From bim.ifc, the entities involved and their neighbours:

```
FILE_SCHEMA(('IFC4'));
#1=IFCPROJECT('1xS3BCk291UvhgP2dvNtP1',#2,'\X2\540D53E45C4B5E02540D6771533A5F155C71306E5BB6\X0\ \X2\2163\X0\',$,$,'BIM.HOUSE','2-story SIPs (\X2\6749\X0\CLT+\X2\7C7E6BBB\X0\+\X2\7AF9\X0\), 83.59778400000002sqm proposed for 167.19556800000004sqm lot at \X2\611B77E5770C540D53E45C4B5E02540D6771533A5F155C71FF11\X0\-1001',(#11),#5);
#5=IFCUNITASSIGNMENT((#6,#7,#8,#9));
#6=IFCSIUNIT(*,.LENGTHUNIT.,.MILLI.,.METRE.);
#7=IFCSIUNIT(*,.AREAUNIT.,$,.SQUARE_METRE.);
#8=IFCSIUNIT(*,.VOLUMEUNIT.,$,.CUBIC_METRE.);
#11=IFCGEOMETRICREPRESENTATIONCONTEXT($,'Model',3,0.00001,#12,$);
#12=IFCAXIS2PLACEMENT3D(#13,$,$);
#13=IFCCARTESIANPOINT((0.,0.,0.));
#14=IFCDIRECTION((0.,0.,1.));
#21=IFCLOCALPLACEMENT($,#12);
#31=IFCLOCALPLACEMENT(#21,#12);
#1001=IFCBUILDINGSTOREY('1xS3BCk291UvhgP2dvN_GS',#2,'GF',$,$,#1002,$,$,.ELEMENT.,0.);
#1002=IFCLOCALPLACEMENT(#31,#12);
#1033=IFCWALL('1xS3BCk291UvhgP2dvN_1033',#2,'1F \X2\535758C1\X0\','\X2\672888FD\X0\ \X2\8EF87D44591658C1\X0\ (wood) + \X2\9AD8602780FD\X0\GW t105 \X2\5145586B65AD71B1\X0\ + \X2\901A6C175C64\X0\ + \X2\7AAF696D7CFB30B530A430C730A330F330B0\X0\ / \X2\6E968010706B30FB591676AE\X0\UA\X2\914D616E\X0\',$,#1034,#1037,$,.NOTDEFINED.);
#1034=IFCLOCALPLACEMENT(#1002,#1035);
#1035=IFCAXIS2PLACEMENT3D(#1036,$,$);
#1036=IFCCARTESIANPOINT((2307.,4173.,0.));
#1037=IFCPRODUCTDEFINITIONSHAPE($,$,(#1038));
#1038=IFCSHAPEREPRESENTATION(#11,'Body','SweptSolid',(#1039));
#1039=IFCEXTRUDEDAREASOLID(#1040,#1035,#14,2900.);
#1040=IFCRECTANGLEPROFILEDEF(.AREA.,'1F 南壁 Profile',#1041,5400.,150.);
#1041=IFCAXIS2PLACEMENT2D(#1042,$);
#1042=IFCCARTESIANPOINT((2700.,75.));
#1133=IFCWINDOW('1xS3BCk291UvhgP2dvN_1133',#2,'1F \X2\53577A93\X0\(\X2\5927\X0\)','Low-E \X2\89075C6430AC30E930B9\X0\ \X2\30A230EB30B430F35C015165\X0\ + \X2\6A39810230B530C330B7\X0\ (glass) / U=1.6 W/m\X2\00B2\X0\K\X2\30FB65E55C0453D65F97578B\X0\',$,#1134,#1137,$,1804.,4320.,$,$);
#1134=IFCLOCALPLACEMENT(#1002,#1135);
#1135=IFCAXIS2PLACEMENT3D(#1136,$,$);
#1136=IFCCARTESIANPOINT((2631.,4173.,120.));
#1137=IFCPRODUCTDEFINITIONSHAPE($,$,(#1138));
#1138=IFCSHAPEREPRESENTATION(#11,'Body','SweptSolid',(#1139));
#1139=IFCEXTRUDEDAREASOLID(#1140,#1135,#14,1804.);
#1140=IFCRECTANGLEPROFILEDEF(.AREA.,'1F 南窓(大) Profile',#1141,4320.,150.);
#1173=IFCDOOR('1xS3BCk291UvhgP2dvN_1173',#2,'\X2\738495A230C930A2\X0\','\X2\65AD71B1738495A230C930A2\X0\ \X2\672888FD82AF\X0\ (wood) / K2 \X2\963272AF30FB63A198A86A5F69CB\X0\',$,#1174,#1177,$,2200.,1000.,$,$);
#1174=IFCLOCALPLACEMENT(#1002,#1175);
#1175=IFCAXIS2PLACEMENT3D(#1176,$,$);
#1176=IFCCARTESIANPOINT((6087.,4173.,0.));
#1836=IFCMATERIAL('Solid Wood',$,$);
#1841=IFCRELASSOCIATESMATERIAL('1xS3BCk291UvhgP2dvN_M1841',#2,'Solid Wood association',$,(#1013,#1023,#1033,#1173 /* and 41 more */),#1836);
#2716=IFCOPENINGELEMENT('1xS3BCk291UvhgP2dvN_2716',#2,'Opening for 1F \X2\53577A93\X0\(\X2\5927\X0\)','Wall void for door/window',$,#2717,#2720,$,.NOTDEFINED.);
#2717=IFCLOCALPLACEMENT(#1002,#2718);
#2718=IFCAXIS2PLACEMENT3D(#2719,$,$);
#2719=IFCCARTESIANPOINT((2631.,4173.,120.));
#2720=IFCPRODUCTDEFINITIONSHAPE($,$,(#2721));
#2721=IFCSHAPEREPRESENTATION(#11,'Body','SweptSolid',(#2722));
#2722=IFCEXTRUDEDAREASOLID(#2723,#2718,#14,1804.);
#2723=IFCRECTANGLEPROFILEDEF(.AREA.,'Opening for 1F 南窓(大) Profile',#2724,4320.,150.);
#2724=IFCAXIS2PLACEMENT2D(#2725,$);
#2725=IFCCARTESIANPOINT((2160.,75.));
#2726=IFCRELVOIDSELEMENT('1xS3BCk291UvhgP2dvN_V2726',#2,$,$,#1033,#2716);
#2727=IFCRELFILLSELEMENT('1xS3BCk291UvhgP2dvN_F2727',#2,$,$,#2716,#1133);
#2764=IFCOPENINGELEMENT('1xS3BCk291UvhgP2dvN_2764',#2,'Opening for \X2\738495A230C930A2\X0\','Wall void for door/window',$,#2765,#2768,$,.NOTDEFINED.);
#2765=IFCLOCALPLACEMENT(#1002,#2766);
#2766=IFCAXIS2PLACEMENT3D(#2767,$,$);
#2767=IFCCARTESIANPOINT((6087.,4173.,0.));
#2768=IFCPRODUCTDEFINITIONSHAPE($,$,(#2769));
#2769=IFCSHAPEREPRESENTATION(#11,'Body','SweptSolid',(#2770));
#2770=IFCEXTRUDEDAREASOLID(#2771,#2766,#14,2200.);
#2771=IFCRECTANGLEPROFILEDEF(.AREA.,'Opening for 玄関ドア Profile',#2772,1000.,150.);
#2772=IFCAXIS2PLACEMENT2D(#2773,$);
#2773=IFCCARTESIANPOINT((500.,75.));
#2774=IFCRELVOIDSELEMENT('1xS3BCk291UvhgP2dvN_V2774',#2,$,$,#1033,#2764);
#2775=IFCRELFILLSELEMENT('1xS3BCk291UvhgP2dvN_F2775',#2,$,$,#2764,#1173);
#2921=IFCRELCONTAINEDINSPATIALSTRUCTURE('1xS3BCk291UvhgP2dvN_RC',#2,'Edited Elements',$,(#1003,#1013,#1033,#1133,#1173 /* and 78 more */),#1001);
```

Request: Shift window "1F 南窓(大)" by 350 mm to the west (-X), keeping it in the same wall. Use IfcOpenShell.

```python
import ifcopenshell
import ifcopenshell.api.geometry
import ifcopenshell.util.placement
import ifcopenshell.util.unit

model = ifcopenshell.open("bim.ifc")
unit_scale = ifcopenshell.util.unit.calculate_unit_scale(model)

window = model.by_guid("1xS3BCk291UvhgP2dvN_1133")
opening = window.FillsVoids[0].RelatingOpeningElement
wall = opening.VoidsElements[0].RelatingBuildingElement

wall_matrix = ifcopenshell.util.placement.get_local_placement(wall.ObjectPlacement)
shift = wall_matrix[:3, 0] * -0.35 / unit_scale
before = ifcopenshell.util.placement.get_local_placement(window.ObjectPlacement)[:3, 3].copy()

# The window is not placed relative to its opening, so move both.
for product in (opening, window):
    matrix = ifcopenshell.util.placement.get_local_placement(product.ObjectPlacement)
    matrix[:3, 3] += shift
    ifcopenshell.api.geometry.edit_object_placement(model, product=product, matrix=matrix, is_si=False)

after = ifcopenshell.util.placement.get_local_placement(window.ObjectPlacement)[:3, 3]
print("window moved by", (after - before).round(3) + 0.0)

model.write("bim_v2.ifc")
```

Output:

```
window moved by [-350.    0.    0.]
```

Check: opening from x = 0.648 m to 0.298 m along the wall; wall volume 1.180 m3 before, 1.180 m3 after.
